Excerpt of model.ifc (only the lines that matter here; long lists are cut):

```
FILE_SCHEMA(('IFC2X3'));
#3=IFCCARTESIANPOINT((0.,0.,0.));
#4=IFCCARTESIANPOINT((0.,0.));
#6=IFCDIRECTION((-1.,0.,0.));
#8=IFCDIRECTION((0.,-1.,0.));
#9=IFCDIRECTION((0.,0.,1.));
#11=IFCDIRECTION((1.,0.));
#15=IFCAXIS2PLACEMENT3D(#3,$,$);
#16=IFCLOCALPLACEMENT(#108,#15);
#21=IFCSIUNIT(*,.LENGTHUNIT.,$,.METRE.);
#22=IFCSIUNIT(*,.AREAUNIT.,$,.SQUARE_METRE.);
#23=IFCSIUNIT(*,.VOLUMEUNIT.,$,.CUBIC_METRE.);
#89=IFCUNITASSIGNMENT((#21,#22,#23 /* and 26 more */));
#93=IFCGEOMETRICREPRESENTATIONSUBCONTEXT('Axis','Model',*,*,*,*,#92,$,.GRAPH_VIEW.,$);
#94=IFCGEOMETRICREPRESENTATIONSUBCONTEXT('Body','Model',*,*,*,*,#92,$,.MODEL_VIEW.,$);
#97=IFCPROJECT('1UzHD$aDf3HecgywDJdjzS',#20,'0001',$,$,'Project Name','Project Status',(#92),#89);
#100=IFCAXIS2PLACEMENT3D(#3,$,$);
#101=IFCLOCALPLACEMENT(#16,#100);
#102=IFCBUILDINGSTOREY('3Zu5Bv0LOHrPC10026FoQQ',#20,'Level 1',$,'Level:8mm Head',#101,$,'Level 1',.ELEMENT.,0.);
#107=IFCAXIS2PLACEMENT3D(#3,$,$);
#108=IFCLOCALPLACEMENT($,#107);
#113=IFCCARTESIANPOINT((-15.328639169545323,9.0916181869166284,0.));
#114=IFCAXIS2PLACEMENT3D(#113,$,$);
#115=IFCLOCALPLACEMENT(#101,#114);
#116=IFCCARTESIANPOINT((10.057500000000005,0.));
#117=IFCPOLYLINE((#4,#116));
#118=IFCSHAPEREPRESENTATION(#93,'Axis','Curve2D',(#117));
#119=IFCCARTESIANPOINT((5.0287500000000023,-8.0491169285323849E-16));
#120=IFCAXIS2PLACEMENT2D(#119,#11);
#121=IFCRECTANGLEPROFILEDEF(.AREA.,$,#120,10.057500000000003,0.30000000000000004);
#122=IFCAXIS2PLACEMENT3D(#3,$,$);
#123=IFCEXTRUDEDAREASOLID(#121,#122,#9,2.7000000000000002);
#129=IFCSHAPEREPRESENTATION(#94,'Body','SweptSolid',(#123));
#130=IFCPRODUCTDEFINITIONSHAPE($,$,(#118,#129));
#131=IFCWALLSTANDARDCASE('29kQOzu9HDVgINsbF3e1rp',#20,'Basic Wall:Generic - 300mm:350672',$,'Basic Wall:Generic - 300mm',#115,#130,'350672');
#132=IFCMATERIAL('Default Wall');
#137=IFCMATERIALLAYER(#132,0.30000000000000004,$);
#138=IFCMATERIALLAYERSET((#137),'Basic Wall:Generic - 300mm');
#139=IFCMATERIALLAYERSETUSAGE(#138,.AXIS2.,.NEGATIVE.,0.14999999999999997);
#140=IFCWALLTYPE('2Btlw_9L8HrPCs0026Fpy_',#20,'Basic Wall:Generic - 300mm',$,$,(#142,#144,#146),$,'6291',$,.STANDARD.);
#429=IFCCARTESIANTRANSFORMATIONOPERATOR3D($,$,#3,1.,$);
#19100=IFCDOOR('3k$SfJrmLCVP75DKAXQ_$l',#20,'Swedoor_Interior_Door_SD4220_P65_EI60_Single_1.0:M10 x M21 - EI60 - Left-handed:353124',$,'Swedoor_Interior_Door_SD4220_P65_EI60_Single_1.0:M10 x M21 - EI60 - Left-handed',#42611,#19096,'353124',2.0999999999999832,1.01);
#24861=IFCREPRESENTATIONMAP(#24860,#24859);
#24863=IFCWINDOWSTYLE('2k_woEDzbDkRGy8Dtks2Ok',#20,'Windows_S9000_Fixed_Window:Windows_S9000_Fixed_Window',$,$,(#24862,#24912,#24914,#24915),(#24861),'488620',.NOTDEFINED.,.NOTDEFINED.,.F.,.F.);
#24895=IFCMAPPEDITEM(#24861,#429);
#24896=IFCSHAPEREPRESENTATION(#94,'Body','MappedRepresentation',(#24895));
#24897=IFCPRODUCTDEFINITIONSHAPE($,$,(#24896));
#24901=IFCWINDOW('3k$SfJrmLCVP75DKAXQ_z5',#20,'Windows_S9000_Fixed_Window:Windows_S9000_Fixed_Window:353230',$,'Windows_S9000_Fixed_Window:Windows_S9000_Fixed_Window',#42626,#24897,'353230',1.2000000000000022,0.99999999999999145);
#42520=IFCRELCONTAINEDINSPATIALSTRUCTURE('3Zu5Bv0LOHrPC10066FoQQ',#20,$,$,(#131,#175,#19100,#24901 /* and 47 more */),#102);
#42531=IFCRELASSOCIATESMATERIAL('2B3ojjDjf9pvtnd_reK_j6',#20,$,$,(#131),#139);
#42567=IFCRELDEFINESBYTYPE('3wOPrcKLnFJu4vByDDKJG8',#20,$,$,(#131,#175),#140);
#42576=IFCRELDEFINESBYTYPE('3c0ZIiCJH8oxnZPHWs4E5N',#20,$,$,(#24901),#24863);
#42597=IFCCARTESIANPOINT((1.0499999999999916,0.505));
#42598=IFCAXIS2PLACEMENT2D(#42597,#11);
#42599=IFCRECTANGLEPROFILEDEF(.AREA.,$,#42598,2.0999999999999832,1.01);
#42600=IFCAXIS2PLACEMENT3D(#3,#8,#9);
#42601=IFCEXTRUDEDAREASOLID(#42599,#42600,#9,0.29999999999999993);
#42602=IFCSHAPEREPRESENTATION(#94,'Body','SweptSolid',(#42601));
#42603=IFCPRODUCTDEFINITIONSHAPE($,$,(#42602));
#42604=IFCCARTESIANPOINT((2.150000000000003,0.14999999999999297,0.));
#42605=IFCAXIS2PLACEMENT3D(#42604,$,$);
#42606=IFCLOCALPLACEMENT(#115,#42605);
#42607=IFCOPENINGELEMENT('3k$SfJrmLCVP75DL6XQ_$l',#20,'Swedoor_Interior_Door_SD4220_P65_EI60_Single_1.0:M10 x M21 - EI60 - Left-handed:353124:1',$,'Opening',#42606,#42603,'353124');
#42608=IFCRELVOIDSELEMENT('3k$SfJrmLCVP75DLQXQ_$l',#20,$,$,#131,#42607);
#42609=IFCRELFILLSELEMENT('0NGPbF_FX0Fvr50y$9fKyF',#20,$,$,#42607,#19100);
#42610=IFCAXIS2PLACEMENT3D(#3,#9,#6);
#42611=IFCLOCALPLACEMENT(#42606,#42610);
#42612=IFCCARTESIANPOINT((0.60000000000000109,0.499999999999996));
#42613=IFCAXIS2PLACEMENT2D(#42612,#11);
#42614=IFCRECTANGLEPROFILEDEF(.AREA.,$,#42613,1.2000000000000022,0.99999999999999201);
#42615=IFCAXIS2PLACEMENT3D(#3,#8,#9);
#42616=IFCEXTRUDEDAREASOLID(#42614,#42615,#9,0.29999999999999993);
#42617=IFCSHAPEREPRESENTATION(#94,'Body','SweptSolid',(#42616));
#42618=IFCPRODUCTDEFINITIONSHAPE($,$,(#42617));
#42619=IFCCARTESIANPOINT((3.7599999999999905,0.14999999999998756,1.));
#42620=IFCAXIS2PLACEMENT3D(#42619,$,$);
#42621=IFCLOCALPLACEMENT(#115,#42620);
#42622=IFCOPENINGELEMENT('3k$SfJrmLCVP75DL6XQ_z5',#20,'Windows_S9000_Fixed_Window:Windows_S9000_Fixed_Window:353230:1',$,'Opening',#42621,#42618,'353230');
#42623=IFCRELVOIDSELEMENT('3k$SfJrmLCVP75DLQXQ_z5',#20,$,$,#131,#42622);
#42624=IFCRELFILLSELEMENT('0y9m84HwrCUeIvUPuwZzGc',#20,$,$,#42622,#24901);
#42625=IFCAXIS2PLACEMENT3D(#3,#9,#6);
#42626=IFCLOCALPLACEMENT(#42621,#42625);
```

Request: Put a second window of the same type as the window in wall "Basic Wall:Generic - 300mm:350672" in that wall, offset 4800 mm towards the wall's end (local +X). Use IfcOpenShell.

```python
import ifcopenshell
import ifcopenshell.api.feature
import ifcopenshell.api.geometry
import ifcopenshell.api.root
import ifcopenshell.geom
import ifcopenshell.util.element
import ifcopenshell.util.placement
import ifcopenshell.util.shape
import ifcopenshell.util.unit

model = ifcopenshell.open("model.ifc")
unit_scale = ifcopenshell.util.unit.calculate_unit_scale(model)
settings = ifcopenshell.geom.settings()


def volume(element):
    """Net volume in cubic metres, openings subtracted."""
    shape = ifcopenshell.geom.create_shape(settings, element)
    return ifcopenshell.util.shape.get_volume(shape.geometry)


def reuse_history(source, copy):
    """copy_class also copies each property set's owner history, people and application; keep the originals."""
    for rel in copy.IsDefinedBy:
        if rel.is_a("IfcRelDefinesByProperties") and (history := rel.RelatingPropertyDefinition.OwnerHistory):
            rel.RelatingPropertyDefinition.OwnerHistory = source.OwnerHistory
            ifcopenshell.util.element.remove_deep2(model, history)


window = model.by_guid("3k$SfJrmLCVP75DKAXQ_z5")
opening = window.FillsVoids[0].RelatingOpeningElement
wall = opening.VoidsElements[0].RelatingBuildingElement
before = volume(wall)
shift = ifcopenshell.util.placement.get_local_placement(wall.ObjectPlacement)[:3, 0] * 4.8 / unit_scale

# copy_class copies the void relationship, type, container and properties, but no geometry.
new_opening = ifcopenshell.api.root.copy_class(model, product=opening)
new_opening.Representation = ifcopenshell.util.element.copy_deep(
    model, opening.Representation, exclude=["IfcGeometricRepresentationContext", "IfcRepresentationMap"]
)
new_opening.Name = "Windows_S9000_Fixed_Window:Windows_S9000_Fixed_Window"
new_opening.Tag = None
new_window = ifcopenshell.api.root.copy_class(model, product=window)
new_window.Representation = ifcopenshell.util.element.copy_deep(
    model, window.Representation, exclude=["IfcGeometricRepresentationContext", "IfcRepresentationMap"]
)
new_window.Name = "Windows_S9000_Fixed_Window:Windows_S9000_Fixed_Window"
new_window.Tag = None
reuse_history(window, new_window)
fills = ifcopenshell.api.feature.add_filling(model, opening=new_opening, element=new_window)
fills.OwnerHistory = new_window.OwnerHistory  # required in IFC2X3

for old, new in ((opening, new_opening), (window, new_window)):
    matrix = ifcopenshell.util.placement.get_local_placement(old.ObjectPlacement)
    matrix[:3, 3] += shift
    ifcopenshell.api.geometry.edit_object_placement(model, product=new, matrix=matrix, is_si=False)

after = volume(wall)

print(f"wall volume {before:.3f} -> {after:.3f} m3")

model.write("model-out.ifc")
```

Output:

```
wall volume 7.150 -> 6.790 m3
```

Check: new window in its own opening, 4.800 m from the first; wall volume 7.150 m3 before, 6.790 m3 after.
